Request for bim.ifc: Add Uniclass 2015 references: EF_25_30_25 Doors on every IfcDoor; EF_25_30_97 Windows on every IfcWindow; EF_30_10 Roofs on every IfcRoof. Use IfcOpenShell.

First a look at what the model holds.

```python
import ifcopenshell

model = ifcopenshell.open("bim.ifc")
print(model.schema)
print("classifications:", [c.Name for c in model.by_type("IfcClassification")])
for ifc_class in ("IfcDoor", "IfcRoof", "IfcStair", "IfcWall", "IfcWindow"):
    print(ifc_class, len(model.by_type(ifc_class)))
```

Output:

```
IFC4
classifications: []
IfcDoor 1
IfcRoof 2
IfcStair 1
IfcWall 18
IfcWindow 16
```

```python
import ifcopenshell
import ifcopenshell.api.classification

model = ifcopenshell.open("bim.ifc")

system = ifcopenshell.api.classification.add_classification(model, classification="Uniclass 2015")

codes = {
    "IfcDoor": ("EF_25_30_25", "Doors"),
    "IfcWindow": ("EF_25_30_97", "Windows"),
    "IfcRoof": ("EF_30_10", "Roofs"),
}
for ifc_class, (code, name) in codes.items():
    products = model.by_type(ifc_class)
    ifcopenshell.api.classification.add_reference(
        model, products=products, classification=system, identification=code, name=name
    )
    print(code, len(products))

model.write("bim_rev.ifc")
```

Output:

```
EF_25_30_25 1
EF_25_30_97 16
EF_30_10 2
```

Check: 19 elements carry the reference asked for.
